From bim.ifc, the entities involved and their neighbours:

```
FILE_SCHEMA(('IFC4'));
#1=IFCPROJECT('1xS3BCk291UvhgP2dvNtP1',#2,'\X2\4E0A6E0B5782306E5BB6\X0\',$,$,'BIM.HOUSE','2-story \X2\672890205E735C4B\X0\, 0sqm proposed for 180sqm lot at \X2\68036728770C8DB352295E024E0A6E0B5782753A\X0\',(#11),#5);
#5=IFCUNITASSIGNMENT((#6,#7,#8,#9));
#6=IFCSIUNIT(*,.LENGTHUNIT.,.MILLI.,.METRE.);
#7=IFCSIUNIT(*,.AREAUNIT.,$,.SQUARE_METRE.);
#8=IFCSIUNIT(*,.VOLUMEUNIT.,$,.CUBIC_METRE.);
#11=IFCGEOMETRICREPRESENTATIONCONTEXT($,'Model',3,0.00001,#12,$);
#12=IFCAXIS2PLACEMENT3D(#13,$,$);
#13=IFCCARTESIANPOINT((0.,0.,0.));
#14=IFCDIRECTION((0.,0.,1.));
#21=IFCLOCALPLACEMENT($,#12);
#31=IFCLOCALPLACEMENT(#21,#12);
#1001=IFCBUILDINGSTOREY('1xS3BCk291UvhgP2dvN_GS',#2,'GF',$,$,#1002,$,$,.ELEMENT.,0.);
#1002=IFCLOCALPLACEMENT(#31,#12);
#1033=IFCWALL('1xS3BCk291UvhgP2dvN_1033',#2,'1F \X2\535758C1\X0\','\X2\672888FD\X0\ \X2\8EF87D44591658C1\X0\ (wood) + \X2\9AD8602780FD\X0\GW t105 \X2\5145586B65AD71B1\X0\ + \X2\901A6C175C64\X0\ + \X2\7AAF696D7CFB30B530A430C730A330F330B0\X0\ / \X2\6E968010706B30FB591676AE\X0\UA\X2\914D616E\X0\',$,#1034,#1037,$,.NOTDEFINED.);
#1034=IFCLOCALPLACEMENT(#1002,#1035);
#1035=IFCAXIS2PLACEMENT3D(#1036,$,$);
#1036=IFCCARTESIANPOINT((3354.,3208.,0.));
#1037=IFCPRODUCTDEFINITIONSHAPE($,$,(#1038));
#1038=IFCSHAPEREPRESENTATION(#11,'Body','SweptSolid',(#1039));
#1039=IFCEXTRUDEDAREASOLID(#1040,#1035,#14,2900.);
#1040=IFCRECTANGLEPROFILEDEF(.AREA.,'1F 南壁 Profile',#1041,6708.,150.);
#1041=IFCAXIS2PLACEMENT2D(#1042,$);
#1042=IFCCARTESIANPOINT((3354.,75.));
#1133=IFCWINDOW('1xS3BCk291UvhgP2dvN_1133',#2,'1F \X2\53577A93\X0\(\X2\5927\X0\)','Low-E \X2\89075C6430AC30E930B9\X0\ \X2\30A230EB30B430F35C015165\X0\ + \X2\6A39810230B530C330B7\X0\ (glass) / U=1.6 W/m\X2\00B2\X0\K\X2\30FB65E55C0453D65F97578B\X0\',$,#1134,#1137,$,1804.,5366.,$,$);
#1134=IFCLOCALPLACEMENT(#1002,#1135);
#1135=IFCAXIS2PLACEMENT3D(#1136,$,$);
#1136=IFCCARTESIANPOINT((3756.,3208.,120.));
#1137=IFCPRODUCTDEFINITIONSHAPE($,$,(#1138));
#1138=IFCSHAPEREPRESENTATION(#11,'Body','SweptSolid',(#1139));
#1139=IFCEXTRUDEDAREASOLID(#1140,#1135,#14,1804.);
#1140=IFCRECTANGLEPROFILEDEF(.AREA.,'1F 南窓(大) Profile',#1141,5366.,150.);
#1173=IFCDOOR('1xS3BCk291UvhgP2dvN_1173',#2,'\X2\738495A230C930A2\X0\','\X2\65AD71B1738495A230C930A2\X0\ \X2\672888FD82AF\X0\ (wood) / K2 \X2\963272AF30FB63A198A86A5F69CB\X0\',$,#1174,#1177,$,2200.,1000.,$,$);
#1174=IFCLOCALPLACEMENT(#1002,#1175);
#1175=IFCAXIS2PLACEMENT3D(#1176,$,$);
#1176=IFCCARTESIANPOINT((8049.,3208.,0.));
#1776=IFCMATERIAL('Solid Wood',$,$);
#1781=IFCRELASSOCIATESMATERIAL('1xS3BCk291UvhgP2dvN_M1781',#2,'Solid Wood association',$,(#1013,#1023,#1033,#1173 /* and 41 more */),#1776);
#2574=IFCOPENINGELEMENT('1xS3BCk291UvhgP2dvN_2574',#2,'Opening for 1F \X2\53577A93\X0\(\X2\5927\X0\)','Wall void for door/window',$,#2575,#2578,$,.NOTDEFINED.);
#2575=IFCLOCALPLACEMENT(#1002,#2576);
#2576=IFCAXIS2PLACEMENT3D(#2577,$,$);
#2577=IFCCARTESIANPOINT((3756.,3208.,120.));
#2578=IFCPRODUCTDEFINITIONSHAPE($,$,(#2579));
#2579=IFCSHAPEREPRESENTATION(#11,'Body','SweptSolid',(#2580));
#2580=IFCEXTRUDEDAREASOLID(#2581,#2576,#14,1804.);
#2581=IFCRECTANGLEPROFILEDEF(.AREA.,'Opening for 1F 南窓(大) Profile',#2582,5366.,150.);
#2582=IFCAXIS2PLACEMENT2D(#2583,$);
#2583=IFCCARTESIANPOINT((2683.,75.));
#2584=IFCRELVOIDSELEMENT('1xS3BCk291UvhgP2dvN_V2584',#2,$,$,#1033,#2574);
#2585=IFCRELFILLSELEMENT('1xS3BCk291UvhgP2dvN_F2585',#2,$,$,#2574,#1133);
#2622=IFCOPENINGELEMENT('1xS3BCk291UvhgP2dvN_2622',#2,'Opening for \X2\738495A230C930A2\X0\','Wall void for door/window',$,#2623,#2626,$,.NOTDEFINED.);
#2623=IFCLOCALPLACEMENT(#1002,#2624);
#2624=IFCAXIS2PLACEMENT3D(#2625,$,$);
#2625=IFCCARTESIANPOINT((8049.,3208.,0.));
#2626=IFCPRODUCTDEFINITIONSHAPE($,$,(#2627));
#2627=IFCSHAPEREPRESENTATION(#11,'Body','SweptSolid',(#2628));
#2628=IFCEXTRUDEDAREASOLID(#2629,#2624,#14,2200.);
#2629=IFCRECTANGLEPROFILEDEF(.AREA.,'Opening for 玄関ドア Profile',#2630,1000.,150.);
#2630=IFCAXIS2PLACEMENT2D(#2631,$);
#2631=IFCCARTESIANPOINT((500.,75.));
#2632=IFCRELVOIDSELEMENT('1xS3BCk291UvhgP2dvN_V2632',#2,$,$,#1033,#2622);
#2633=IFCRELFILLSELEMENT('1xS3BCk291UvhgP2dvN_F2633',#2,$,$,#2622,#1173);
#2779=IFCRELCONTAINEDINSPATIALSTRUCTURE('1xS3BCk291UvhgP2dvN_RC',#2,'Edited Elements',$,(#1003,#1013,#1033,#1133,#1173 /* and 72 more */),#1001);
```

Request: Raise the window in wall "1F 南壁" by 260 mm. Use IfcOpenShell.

```python
import numpy as np
import ifcopenshell
import ifcopenshell.api.geometry
import ifcopenshell.util.placement
import ifcopenshell.util.unit

model = ifcopenshell.open("bim.ifc")
unit_scale = ifcopenshell.util.unit.calculate_unit_scale(model)

window = model.by_guid("1xS3BCk291UvhgP2dvN_1133")
opening = window.FillsVoids[0].RelatingOpeningElement
dz = 0.26 / unit_scale

shift = np.array([0.0, 0.0, dz])
# The window is not placed relative to its opening, so move both.
for product in (opening, window):
    matrix = ifcopenshell.util.placement.get_local_placement(product.ObjectPlacement)
    matrix[:3, 3] += shift
    ifcopenshell.api.geometry.edit_object_placement(model, product=product, matrix=matrix, is_si=False)

print(f"moved by {dz * unit_scale:+.3f} m")

model.write("bim-out.ifc")
```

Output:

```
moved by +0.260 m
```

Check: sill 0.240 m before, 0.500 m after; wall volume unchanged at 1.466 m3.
